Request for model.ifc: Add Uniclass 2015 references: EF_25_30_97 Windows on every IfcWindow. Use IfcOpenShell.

First a look at what the model holds.

```python
import ifcopenshell

model = ifcopenshell.open("model.ifc")
print(model.schema)
print("classifications:", [c.Name for c in model.by_type("IfcClassification")])
for ifc_class in ("IfcDoor", "IfcRoof", "IfcStair", "IfcWall", "IfcWindow"):
    print(ifc_class, len(model.by_type(ifc_class)))
```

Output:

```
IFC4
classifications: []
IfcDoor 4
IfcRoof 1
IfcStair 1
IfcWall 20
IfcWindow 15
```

```python
import ifcopenshell
import ifcopenshell.api.classification

model = ifcopenshell.open("model.ifc")

system = ifcopenshell.api.classification.add_classification(model, classification="Uniclass 2015")

codes = {
    "IfcWindow": ("EF_25_30_97", "Windows"),
}
for ifc_class, (code, name) in codes.items():
    products = model.by_type(ifc_class)
    ifcopenshell.api.classification.add_reference(
        model, products=products, classification=system, identification=code, name=name
    )
    print(code, len(products))

model.write("model_edited.ifc")
```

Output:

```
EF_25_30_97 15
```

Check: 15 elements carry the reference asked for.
